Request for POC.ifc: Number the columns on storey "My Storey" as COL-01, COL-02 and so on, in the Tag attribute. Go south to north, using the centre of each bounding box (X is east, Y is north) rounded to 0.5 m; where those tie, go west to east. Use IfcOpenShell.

First a look at what the model holds.

```python
import ifcopenshell
import ifcopenshell.util.element
import ifcopenshell.util.placement

model = ifcopenshell.open("POC.ifc")
print(model.schema)
storey = next(s for s in model.by_type("IfcBuildingStorey") if s.Name == "My Storey")
columns = [e for e in ifcopenshell.util.element.get_decomposition(storey) if e.is_a("IfcColumn")]
for e in sorted(columns, key=lambda e: e.id()):
    origin = ifcopenshell.util.placement.get_local_placement(e.ObjectPlacement)[:3, 3]
    print(e.id(), e.Tag, e.Name, origin.round(2) + 0.0, sep=" | ")
```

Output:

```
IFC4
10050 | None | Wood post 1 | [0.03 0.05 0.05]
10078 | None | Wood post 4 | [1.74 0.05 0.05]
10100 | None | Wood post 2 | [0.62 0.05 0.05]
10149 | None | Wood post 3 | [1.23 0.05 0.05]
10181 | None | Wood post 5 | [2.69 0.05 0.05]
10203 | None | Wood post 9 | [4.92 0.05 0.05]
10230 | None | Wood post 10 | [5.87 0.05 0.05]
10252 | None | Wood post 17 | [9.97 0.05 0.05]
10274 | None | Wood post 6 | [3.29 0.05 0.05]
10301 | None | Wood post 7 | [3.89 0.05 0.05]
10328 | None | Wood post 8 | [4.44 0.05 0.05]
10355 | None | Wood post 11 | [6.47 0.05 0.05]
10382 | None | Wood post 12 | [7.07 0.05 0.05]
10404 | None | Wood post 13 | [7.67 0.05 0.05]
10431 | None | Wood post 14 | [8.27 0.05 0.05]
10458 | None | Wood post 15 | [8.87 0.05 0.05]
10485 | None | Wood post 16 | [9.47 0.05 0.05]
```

```python
import ifcopenshell
import ifcopenshell.geom
import ifcopenshell.util.element
import ifcopenshell.util.shape

model = ifcopenshell.open("POC.ifc")
settings = ifcopenshell.geom.settings()
settings.set("use-world-coords", True)


def centre(element):
    shape = ifcopenshell.geom.create_shape(settings, element)
    return ifcopenshell.util.shape.get_bbox_centroid(shape.geometry)


storey = next(s for s in model.by_type("IfcBuildingStorey") if s.Name == "My Storey")
columns = [e for e in ifcopenshell.util.element.get_decomposition(storey) if e.is_a("IfcColumn")]

# Insertion points can sit at a corner or the storey origin, so sort by the geometry (in metres).
centres = {e: centre(e) for e in columns}
columns.sort(key=lambda e: (round(centres[e][1] / 0.5), centres[e][0]))

for i, e in enumerate(columns, start=1):
    number = f"COL-{i:02d}"
    e.Tag = number
    print(e.id(), number)

model.write("POC_updated.ifc")
```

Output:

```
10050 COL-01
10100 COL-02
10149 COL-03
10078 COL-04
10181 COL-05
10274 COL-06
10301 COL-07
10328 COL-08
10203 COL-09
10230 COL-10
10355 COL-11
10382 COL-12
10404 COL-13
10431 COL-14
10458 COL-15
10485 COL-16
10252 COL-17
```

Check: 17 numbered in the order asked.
